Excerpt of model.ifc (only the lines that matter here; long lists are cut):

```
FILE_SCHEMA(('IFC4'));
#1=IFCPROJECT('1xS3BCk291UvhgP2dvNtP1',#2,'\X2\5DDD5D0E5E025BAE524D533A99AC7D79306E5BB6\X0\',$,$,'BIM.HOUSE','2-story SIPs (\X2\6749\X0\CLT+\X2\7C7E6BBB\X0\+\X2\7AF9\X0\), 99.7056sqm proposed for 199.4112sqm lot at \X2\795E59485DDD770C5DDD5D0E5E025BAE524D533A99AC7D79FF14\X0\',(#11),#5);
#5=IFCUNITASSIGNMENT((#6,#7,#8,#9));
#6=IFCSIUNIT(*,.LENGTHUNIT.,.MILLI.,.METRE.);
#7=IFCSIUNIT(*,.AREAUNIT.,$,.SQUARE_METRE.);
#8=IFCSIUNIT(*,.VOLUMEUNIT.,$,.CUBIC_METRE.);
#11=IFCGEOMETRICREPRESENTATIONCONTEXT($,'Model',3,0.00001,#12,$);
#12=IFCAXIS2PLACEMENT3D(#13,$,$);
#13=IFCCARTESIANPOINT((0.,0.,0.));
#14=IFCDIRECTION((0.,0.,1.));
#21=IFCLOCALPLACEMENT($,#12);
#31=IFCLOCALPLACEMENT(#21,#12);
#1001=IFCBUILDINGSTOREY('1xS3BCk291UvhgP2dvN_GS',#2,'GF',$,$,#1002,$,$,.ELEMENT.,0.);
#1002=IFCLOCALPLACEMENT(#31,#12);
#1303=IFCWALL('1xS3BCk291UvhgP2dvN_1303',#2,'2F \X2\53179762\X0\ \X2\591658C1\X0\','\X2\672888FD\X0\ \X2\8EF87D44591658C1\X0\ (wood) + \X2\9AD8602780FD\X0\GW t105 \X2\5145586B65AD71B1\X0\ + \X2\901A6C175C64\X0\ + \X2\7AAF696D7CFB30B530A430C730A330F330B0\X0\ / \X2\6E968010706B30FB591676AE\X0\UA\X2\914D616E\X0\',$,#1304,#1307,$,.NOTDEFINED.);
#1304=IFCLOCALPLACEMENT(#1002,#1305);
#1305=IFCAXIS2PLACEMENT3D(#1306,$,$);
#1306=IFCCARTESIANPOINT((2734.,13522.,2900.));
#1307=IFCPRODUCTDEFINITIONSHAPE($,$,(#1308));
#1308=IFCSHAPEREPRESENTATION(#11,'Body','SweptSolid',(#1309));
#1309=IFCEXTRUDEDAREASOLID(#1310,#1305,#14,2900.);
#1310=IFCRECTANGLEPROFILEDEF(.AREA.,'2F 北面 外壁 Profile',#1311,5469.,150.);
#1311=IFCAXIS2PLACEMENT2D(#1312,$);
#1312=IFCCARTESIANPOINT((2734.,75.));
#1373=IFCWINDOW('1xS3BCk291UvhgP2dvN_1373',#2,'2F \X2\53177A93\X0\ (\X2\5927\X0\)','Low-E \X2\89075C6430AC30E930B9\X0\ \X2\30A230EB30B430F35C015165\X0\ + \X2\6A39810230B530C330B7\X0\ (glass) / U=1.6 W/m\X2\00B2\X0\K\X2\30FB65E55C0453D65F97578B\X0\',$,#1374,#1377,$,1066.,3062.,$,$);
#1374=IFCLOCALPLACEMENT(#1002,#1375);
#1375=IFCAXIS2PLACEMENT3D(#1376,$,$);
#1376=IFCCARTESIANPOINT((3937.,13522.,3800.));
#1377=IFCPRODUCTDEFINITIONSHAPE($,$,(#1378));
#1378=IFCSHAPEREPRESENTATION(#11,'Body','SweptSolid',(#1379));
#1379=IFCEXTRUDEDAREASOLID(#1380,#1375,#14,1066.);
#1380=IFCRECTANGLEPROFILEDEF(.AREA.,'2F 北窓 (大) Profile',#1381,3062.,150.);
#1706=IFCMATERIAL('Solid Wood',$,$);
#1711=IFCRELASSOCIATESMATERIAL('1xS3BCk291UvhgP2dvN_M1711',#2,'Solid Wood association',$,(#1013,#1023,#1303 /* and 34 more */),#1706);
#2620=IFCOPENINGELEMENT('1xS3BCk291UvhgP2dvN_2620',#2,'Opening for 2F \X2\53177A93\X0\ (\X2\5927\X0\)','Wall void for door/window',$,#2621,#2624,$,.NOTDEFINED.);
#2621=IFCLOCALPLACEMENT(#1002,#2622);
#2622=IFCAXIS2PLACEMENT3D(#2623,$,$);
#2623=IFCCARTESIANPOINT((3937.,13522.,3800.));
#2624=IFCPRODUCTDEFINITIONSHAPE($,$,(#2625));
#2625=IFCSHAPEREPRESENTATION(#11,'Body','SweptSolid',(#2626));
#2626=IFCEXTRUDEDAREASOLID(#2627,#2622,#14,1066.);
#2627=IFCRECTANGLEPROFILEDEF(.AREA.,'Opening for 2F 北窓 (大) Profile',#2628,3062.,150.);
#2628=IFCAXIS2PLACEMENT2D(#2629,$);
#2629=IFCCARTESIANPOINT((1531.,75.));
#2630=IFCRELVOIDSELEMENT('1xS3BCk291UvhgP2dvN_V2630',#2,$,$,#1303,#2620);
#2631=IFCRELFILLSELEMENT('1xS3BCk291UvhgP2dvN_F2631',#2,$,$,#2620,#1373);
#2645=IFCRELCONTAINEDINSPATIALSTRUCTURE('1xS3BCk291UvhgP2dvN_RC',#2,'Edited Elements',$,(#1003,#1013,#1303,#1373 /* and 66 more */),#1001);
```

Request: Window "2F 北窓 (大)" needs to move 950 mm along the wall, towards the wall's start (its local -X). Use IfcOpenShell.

```python
import ifcopenshell
import ifcopenshell.api.geometry
import ifcopenshell.util.placement
import ifcopenshell.util.unit

model = ifcopenshell.open("model.ifc")
unit_scale = ifcopenshell.util.unit.calculate_unit_scale(model)

window = model.by_guid("1xS3BCk291UvhgP2dvN_1373")
opening = window.FillsVoids[0].RelatingOpeningElement
wall = opening.VoidsElements[0].RelatingBuildingElement

wall_matrix = ifcopenshell.util.placement.get_local_placement(wall.ObjectPlacement)
shift = wall_matrix[:3, 0] * -0.95 / unit_scale
before = ifcopenshell.util.placement.get_local_placement(window.ObjectPlacement)[:3, 3].copy()

# The window is not placed relative to its opening, so move both.
for product in (opening, window):
    matrix = ifcopenshell.util.placement.get_local_placement(product.ObjectPlacement)
    matrix[:3, 3] += shift
    ifcopenshell.api.geometry.edit_object_placement(model, product=product, matrix=matrix, is_si=False)

after = ifcopenshell.util.placement.get_local_placement(window.ObjectPlacement)[:3, 3]
print("window moved by", (after - before).round(3) + 0.0)

model.write("model_edited.ifc")
```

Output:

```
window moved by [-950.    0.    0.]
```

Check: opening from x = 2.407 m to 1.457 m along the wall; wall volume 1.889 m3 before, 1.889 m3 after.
